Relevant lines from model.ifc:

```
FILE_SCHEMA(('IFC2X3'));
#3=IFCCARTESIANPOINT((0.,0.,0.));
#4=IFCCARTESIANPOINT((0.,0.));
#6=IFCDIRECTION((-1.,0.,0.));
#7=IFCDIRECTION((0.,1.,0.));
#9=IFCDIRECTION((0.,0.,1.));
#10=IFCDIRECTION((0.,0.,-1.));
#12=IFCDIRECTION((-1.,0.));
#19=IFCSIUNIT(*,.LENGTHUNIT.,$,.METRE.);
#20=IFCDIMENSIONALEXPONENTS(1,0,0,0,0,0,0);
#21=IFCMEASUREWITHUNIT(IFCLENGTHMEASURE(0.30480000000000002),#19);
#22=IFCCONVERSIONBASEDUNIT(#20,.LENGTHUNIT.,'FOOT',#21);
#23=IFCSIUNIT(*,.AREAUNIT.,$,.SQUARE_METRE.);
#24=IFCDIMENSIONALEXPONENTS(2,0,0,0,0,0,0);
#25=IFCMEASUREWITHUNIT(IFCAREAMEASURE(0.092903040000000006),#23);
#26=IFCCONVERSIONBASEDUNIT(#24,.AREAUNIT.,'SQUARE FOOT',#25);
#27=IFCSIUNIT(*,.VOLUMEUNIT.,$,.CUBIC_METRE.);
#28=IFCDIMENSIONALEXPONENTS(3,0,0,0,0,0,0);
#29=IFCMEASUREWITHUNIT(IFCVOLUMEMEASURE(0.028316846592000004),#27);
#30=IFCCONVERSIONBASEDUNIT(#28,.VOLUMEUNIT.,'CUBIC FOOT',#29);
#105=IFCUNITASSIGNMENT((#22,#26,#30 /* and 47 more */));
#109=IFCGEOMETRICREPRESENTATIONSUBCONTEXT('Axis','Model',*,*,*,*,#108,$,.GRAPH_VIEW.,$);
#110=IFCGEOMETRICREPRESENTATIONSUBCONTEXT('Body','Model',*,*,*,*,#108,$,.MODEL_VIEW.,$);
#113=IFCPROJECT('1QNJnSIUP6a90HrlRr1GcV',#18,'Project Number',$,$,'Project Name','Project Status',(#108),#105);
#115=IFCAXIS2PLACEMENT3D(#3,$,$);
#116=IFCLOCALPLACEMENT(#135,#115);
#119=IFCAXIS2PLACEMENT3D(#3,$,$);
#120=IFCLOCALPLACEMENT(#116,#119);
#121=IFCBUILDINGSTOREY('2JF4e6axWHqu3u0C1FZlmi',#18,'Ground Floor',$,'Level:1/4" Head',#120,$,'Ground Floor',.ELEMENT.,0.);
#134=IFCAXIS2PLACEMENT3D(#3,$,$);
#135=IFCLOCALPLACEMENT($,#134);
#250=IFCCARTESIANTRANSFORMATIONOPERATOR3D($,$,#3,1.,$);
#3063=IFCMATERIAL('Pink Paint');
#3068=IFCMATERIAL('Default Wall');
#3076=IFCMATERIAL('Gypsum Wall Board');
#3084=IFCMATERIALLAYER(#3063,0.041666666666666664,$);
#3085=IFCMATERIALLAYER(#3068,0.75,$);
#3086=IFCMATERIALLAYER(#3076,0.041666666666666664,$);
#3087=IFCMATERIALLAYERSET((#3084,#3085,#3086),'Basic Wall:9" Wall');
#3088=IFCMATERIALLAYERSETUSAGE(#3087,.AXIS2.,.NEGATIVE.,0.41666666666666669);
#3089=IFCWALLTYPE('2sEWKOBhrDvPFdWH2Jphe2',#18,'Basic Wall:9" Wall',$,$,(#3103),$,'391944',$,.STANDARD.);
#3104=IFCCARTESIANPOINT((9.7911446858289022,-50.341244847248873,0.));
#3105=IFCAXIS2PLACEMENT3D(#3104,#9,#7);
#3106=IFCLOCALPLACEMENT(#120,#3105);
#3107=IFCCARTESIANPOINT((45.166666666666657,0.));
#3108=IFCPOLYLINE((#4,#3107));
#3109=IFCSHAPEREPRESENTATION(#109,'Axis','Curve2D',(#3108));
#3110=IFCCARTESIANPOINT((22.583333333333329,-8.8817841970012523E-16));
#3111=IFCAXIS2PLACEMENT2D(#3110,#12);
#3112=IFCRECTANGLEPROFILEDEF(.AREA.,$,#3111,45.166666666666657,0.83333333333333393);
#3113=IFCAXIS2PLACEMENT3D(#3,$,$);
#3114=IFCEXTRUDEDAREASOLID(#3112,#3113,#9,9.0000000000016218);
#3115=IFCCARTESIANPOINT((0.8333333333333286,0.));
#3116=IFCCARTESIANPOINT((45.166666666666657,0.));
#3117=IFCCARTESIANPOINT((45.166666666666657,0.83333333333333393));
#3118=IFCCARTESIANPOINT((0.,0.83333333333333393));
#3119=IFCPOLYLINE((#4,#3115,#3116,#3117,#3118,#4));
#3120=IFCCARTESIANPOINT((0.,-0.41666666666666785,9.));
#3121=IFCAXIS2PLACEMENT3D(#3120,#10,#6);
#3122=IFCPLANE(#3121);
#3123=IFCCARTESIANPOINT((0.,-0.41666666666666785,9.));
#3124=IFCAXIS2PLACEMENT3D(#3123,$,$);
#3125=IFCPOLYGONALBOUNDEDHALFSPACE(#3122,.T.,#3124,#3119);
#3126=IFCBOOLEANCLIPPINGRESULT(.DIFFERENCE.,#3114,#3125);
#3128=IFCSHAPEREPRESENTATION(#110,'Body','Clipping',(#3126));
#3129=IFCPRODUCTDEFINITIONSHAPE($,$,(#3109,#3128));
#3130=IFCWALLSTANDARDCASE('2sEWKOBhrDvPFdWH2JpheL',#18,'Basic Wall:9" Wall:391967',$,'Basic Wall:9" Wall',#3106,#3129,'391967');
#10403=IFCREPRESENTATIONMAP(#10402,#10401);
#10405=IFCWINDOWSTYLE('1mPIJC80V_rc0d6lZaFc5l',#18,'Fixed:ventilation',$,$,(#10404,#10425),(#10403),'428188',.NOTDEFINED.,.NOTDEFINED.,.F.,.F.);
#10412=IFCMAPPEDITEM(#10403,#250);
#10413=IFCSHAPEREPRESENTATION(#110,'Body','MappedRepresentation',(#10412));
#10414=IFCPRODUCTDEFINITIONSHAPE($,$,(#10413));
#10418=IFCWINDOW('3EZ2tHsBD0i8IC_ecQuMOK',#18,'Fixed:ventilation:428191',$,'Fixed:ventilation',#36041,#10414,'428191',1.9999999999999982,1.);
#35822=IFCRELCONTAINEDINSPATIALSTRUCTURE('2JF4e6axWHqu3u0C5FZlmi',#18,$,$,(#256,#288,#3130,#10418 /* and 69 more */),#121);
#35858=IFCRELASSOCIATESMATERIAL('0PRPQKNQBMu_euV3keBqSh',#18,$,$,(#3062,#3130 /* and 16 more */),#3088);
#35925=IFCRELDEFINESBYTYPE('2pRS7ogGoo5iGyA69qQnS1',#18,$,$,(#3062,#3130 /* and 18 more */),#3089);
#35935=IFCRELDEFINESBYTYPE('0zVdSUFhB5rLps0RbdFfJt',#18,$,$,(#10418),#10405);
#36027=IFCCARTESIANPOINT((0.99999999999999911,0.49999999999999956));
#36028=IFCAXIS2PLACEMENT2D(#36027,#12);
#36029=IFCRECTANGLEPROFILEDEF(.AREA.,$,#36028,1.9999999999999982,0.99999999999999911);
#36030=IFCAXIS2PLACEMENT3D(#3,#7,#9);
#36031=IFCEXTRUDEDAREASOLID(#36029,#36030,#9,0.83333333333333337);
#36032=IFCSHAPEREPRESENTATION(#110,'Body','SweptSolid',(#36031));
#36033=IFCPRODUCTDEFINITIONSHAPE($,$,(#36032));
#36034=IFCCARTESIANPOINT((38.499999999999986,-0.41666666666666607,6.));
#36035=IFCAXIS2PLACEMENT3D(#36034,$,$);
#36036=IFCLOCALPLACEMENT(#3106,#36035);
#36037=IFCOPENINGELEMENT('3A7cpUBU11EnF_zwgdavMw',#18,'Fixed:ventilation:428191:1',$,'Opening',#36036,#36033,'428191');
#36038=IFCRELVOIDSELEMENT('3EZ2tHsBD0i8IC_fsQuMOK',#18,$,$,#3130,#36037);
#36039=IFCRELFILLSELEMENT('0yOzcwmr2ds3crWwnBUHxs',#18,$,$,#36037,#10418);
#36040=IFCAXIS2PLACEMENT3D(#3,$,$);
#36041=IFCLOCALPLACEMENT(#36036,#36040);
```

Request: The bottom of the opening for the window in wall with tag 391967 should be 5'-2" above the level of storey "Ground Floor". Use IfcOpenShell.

```python
import numpy as np
import ifcopenshell
import ifcopenshell.api.geometry
import ifcopenshell.geom
import ifcopenshell.util.element
import ifcopenshell.util.placement
import ifcopenshell.util.shape
import ifcopenshell.util.unit

model = ifcopenshell.open("model.ifc")
unit_scale = ifcopenshell.util.unit.calculate_unit_scale(model)

window = model.by_guid("3EZ2tHsBD0i8IC_ecQuMOK")
opening = window.FillsVoids[0].RelatingOpeningElement
storey = ifcopenshell.util.element.get_container(window, ifc_class="IfcBuildingStorey")
level = ifcopenshell.util.placement.get_local_placement(storey.ObjectPlacement)[2, 3]

# The opening's origin need not be at the sill, so measure its lowest point.
shape = ifcopenshell.geom.create_shape(ifcopenshell.geom.settings(), opening)
bottom = ifcopenshell.util.shape.get_shape_bottom_elevation(shape, shape.geometry) / unit_scale
dz = level + 62 * 0.0254 / unit_scale - bottom

shift = np.array([0.0, 0.0, dz])
# The window is placed relative to its opening, so it follows when the opening moves.
matrix = ifcopenshell.util.placement.get_local_placement(opening.ObjectPlacement)
matrix[:3, 3] += shift
ifcopenshell.api.geometry.edit_object_placement(
    model, product=opening, matrix=matrix, is_si=False, should_transform_children=True
)

print(f"moved by {dz * unit_scale:+.3f} m")

model.write("model_edited.ifc")
```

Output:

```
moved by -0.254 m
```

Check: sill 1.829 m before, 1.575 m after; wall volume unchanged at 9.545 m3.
